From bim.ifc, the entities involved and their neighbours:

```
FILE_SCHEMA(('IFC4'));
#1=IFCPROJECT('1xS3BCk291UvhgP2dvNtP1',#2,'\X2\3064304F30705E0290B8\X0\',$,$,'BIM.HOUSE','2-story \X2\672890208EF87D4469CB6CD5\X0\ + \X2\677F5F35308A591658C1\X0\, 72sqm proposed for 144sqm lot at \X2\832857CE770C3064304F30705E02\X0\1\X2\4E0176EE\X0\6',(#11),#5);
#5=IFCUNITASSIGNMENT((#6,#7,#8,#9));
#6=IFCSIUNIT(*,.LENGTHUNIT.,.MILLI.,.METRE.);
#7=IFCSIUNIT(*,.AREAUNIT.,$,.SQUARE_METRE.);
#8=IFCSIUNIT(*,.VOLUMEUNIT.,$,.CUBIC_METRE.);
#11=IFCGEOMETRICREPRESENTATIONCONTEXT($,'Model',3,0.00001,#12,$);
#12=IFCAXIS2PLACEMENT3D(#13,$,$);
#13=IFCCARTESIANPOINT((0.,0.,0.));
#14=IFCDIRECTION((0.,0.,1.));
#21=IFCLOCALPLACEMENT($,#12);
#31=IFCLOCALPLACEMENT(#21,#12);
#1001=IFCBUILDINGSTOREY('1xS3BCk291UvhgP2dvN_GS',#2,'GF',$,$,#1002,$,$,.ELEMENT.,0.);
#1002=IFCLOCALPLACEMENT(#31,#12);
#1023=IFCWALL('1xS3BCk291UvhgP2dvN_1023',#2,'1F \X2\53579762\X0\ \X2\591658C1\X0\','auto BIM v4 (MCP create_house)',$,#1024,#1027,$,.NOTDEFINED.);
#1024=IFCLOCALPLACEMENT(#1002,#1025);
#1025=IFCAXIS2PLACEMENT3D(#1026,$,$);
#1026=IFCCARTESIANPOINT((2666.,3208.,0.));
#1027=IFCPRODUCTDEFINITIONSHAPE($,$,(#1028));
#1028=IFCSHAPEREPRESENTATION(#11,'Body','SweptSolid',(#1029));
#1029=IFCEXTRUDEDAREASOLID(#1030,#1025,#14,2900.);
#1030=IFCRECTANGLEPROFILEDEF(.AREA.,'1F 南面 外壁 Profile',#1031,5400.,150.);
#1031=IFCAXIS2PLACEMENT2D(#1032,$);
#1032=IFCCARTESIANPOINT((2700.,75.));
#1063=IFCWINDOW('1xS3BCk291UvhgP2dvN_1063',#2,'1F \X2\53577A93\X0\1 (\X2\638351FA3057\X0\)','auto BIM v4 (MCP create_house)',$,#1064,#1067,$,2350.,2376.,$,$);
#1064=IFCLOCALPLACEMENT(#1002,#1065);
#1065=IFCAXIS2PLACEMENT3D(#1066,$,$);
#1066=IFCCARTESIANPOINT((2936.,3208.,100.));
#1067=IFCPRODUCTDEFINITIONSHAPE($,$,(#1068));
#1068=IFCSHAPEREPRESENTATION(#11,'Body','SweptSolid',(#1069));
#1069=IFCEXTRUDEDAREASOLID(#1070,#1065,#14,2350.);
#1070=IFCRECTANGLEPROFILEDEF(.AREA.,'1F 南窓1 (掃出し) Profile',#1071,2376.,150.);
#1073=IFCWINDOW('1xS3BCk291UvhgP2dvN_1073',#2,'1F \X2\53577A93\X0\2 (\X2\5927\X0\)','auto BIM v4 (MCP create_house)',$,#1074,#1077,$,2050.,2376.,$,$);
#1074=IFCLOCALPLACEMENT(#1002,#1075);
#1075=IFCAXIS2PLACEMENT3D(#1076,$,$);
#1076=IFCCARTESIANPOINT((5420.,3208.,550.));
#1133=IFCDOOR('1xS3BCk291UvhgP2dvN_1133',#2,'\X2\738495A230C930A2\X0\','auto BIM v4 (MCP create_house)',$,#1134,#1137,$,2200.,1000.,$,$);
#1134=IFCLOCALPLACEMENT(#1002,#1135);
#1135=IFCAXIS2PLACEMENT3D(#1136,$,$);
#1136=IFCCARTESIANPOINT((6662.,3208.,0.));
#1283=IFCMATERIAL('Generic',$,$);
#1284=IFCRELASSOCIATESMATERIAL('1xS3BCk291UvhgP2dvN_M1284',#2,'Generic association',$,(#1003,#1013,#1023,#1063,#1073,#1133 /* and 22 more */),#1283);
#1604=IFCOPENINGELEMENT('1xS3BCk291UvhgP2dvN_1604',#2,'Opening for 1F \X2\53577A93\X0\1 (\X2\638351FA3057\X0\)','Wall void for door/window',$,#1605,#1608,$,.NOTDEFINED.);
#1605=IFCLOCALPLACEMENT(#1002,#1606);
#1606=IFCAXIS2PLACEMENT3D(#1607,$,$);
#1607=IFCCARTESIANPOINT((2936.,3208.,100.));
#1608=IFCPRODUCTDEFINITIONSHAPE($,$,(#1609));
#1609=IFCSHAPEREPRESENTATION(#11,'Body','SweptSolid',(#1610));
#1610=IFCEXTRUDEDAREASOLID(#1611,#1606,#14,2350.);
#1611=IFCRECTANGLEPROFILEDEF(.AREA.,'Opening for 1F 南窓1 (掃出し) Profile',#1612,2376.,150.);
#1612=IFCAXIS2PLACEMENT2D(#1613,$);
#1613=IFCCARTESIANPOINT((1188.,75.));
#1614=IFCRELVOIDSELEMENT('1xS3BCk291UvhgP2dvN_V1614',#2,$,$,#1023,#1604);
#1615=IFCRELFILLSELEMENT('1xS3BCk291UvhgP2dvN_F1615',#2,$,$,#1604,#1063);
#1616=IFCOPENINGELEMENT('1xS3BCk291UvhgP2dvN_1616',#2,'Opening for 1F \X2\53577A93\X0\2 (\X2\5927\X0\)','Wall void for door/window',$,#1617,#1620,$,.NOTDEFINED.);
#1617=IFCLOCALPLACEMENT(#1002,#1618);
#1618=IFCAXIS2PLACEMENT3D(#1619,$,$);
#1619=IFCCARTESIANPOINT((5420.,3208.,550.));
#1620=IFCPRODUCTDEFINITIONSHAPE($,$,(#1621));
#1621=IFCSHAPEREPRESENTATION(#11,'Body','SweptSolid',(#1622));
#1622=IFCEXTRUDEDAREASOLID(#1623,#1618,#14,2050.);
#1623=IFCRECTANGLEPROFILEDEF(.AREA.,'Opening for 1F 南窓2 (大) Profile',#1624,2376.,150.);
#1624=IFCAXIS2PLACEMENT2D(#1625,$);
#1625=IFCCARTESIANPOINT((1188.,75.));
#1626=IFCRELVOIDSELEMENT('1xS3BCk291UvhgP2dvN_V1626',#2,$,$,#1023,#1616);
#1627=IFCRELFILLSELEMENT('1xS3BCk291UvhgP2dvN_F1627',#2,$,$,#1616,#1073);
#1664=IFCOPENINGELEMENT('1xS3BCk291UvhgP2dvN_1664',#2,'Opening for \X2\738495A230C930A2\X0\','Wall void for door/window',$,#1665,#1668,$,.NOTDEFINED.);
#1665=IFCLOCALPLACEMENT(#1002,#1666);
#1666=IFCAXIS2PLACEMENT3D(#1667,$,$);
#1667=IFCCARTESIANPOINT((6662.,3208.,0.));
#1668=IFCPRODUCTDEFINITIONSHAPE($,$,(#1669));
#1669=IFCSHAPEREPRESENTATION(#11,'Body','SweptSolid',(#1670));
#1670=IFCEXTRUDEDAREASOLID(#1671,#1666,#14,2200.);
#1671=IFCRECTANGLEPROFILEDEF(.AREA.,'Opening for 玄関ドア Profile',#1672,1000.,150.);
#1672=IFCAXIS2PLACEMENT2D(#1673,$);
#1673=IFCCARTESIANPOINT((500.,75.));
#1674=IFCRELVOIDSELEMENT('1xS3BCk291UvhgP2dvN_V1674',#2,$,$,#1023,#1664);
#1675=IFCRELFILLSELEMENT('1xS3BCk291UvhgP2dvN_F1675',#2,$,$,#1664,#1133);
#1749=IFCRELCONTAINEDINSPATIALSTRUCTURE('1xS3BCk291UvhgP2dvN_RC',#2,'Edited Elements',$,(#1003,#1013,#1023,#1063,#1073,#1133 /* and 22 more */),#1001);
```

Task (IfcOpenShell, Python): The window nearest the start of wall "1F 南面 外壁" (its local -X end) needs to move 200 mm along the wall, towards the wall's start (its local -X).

```python
import ifcopenshell
import ifcopenshell.api.geometry
import ifcopenshell.util.placement
import ifcopenshell.util.unit

model = ifcopenshell.open("bim.ifc")
unit_scale = ifcopenshell.util.unit.calculate_unit_scale(model)

window = model.by_id(1063)
opening = window.FillsVoids[0].RelatingOpeningElement
wall = opening.VoidsElements[0].RelatingBuildingElement

wall_matrix = ifcopenshell.util.placement.get_local_placement(wall.ObjectPlacement)
shift = wall_matrix[:3, 0] * -0.2 / unit_scale
before = ifcopenshell.util.placement.get_local_placement(window.ObjectPlacement)[:3, 3].copy()

# The window is not placed relative to its opening, so move both.
for product in (opening, window):
    matrix = ifcopenshell.util.placement.get_local_placement(product.ObjectPlacement)
    matrix[:3, 3] += shift
    ifcopenshell.api.geometry.edit_object_placement(model, product=product, matrix=matrix, is_si=False)

after = ifcopenshell.util.placement.get_local_placement(window.ObjectPlacement)[:3, 3]
print("window moved by", (after - before).round(3) + 0.0)

model.write("bim-out.ifc")
```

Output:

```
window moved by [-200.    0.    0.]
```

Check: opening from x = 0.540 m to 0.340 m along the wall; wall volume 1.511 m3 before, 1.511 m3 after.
